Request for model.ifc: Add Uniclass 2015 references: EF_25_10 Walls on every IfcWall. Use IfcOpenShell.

First a look at what the model holds.

```python
import ifcopenshell

model = ifcopenshell.open("model.ifc")
print(model.schema)
print("classifications:", [c.Name for c in model.by_type("IfcClassification")])
for ifc_class in ("IfcDoor", "IfcRoof", "IfcStair", "IfcWall", "IfcWindow"):
    print(ifc_class, len(model.by_type(ifc_class)))
```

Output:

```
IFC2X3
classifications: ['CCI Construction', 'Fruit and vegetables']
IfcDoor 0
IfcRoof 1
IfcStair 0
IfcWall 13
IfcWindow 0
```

```python
import ifcopenshell
import ifcopenshell.api.classification

model = ifcopenshell.open("model.ifc")

# IFC2X3 requires Source and Edition and has no link from the project to the system.
system = model.create_entity("IfcClassification", Source="NBS", Edition="2015", Name="Uniclass 2015")

codes = {
    "IfcWall": ("EF_25_10", "Walls"),
}
for ifc_class, (code, name) in codes.items():
    products = model.by_type(ifc_class)
    ifcopenshell.api.classification.add_reference(
        model, products=products, classification=system, identification=code, name=name
    )
    print(code, len(products))

model.write("model_edited.ifc")
```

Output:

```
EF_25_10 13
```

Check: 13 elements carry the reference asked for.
